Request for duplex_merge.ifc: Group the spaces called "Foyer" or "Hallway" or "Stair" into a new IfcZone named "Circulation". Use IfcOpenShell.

First a look at what the model holds.

```python
import ifcopenshell

model = ifcopenshell.open("duplex_merge.ifc")
print(model.schema)
seen = {}
for space in model.by_type("IfcSpace"):
    seen[space.LongName] = seen.get(space.LongName, 0) + 1
for name, count in sorted(seen.items(), key=str):
    print(count, "x", name)
print("zones:", [z.Name for z in model.by_type("IfcZone")][:20])
```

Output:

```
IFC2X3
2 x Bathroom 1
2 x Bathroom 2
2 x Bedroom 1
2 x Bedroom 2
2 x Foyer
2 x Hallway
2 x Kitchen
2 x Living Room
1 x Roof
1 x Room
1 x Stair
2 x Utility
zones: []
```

```python
import ifcopenshell
import ifcopenshell.api.group
import ifcopenshell.api.root

model = ifcopenshell.open("duplex_merge.ifc")

names = {"Foyer", "Hallway", "Stair"}
spaces = [s for s in model.by_type("IfcSpace") if s.LongName in names]

zone = ifcopenshell.api.root.create_entity(model, ifc_class="IfcZone", name="Circulation")
ifcopenshell.api.group.assign_group(model, products=spaces, group=zone)
print(len(spaces), "spaces in", zone.Name)

model.write("duplex_merge_edited.ifc")
```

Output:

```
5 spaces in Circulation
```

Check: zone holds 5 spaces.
